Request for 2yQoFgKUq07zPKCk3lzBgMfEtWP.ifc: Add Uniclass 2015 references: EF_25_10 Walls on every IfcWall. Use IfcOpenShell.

First a look at what the model holds.

```python
import ifcopenshell

model = ifcopenshell.open("2yQoFgKUq07zPKCk3lzBgMfEtWP.ifc")
print(model.schema)
print("classifications:", [c.Name for c in model.by_type("IfcClassification")])
for ifc_class in ("IfcDoor", "IfcRoof", "IfcStair", "IfcWall", "IfcWindow"):
    print(ifc_class, len(model.by_type(ifc_class)))
```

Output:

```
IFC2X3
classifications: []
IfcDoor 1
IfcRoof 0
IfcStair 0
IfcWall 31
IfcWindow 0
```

```python
import ifcopenshell
import ifcopenshell.api.classification

model = ifcopenshell.open("2yQoFgKUq07zPKCk3lzBgMfEtWP.ifc")

# IFC2X3 requires Source and Edition and has no link from the project to the system.
system = model.create_entity("IfcClassification", Source="NBS", Edition="2015", Name="Uniclass 2015")

codes = {
    "IfcWall": ("EF_25_10", "Walls"),
}
for ifc_class, (code, name) in codes.items():
    products = model.by_type(ifc_class)
    ifcopenshell.api.classification.add_reference(
        model, products=products, classification=system, identification=code, name=name
    )
    print(code, len(products))

model.write("2yQoFgKUq07zPKCk3lzBgMfEtWP_updated.ifc")
```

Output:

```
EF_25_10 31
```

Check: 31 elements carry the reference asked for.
